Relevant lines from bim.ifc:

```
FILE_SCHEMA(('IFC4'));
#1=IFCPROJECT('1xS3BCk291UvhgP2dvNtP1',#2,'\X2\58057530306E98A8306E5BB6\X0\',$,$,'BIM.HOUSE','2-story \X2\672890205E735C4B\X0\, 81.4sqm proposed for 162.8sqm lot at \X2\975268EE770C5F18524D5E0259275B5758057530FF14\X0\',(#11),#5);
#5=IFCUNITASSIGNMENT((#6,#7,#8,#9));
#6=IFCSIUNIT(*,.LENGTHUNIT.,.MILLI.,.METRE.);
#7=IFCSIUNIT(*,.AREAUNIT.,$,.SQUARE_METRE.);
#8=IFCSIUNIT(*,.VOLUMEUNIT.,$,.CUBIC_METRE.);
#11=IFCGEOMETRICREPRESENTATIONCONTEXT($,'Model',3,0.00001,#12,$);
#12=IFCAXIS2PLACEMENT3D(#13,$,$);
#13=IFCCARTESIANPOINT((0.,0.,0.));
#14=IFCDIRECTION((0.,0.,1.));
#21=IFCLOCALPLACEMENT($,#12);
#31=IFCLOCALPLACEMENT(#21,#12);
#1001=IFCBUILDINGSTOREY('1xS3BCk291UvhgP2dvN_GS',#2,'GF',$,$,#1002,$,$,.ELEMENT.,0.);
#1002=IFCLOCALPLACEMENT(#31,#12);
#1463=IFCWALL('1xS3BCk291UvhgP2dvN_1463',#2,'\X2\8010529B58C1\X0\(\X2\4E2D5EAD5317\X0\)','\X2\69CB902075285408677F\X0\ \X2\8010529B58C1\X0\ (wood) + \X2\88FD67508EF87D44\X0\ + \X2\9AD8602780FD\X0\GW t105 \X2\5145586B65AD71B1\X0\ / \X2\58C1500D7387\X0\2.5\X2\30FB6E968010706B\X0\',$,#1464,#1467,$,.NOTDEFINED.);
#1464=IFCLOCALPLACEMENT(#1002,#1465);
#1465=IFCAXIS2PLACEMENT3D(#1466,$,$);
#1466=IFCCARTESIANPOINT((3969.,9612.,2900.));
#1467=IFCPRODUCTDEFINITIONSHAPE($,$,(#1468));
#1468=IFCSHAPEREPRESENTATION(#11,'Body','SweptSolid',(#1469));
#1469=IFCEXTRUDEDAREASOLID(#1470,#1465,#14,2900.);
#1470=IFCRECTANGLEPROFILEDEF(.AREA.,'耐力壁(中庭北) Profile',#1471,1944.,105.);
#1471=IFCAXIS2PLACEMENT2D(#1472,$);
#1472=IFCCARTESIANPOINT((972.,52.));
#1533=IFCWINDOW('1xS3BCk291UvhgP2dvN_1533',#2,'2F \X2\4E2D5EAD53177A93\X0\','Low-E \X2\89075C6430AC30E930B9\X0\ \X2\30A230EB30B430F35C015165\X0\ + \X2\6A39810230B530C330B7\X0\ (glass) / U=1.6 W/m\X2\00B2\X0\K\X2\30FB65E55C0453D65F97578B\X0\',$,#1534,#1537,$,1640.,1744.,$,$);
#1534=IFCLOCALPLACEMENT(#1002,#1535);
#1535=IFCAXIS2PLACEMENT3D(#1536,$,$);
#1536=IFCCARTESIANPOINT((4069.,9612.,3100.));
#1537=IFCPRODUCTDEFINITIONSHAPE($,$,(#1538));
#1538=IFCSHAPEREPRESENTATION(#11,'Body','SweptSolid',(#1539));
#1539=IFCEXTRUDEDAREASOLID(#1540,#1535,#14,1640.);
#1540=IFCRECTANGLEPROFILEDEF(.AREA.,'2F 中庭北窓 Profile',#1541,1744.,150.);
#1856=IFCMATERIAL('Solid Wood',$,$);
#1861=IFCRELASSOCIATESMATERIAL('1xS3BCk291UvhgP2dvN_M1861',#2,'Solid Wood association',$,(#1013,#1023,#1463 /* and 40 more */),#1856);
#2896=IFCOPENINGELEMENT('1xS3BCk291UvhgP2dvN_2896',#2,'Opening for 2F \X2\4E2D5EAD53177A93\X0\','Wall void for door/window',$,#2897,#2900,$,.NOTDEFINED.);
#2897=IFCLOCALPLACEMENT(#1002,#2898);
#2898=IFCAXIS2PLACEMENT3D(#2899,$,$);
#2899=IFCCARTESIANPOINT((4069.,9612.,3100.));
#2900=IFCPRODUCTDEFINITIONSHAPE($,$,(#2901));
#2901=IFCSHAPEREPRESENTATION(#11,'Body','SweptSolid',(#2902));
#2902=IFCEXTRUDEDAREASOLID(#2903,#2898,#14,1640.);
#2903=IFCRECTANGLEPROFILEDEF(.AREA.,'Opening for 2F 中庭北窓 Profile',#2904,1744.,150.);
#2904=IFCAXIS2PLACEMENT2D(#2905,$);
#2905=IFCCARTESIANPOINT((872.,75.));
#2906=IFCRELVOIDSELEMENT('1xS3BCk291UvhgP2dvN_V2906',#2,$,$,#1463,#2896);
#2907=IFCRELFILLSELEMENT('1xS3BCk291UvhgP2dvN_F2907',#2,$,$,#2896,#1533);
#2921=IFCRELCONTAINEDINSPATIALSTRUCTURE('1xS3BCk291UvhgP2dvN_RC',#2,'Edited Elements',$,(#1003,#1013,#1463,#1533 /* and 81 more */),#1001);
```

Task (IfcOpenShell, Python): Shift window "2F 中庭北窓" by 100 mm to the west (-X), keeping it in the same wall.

```python
import ifcopenshell
import ifcopenshell.api.geometry
import ifcopenshell.util.placement

model = ifcopenshell.open("bim.ifc")

window = model.by_guid("1xS3BCk291UvhgP2dvN_1533")
opening = window.FillsVoids[0].RelatingOpeningElement
wall = opening.VoidsElements[0].RelatingBuildingElement

wall_matrix = ifcopenshell.util.placement.get_local_placement(wall.ObjectPlacement)
shift = wall_matrix[:3, 0] * -100.0
before = ifcopenshell.util.placement.get_local_placement(window.ObjectPlacement)[:3, 3].copy()

# The window is not placed relative to its opening, so move both.
for product in (opening, window):
    matrix = ifcopenshell.util.placement.get_local_placement(product.ObjectPlacement)
    matrix[:3, 3] += shift
    ifcopenshell.api.geometry.edit_object_placement(model, product=product, matrix=matrix, is_si=False)

after = ifcopenshell.util.placement.get_local_placement(window.ObjectPlacement)[:3, 3]
print("window moved by", (after - before).round(3) + 0.0)

model.write("bim_v2.ifc")
```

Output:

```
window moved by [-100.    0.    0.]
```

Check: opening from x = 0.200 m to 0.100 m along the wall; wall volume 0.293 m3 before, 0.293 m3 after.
